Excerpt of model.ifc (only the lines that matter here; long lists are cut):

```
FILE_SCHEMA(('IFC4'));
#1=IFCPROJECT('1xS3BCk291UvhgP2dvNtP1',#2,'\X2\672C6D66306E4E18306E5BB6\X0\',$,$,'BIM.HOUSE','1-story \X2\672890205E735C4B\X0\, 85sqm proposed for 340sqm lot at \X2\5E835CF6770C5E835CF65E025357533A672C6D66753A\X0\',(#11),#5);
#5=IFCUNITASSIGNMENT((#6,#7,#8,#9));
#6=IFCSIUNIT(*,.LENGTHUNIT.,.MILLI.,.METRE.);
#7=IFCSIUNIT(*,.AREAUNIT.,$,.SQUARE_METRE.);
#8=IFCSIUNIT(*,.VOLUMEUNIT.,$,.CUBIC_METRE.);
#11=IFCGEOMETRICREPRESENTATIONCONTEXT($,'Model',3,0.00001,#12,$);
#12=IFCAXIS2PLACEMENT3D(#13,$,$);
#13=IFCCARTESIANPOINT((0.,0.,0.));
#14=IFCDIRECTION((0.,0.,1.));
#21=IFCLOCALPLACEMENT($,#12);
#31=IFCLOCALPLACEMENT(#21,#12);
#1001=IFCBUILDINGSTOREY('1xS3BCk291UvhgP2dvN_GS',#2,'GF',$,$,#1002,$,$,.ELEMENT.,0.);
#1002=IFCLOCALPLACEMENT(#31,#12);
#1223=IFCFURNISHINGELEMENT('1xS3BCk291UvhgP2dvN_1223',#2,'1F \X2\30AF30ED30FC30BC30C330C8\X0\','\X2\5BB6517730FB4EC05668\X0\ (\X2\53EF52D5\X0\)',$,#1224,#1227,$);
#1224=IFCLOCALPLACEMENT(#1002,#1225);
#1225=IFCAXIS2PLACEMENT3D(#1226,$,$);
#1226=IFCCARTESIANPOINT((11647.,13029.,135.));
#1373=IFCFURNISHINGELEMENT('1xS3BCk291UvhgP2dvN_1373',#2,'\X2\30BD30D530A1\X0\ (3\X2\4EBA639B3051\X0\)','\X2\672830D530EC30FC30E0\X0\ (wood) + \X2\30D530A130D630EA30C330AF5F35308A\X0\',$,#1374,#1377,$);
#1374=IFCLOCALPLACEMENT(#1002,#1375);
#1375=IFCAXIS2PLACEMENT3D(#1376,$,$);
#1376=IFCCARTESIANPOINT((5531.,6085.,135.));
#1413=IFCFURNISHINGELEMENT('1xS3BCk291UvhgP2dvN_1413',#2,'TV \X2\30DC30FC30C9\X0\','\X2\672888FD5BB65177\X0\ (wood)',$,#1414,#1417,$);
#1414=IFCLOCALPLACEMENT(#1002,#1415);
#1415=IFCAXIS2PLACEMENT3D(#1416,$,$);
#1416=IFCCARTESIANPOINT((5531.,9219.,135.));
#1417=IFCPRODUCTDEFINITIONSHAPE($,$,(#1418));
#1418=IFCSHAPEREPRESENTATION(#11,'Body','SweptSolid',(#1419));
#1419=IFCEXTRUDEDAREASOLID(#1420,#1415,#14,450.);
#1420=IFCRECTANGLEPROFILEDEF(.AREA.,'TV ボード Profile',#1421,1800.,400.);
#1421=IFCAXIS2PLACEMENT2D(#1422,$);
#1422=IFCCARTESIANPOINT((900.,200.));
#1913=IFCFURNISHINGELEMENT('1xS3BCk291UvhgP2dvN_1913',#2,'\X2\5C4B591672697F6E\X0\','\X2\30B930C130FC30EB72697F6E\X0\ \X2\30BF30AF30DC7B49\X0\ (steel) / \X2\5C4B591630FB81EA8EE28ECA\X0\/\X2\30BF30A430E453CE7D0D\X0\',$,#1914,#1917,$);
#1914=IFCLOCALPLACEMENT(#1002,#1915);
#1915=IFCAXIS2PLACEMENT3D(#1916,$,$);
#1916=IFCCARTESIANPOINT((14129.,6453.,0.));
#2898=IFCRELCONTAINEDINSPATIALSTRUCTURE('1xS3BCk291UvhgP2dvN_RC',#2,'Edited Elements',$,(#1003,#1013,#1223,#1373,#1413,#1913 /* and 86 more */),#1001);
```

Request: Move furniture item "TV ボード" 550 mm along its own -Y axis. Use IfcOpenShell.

```python
import ifcopenshell
import ifcopenshell.api.geometry
import ifcopenshell.util.placement
import ifcopenshell.util.unit

model = ifcopenshell.open("model.ifc")
unit_scale = ifcopenshell.util.unit.calculate_unit_scale(model)

item = model.by_guid("1xS3BCk291UvhgP2dvN_1413")
matrix = ifcopenshell.util.placement.get_local_placement(item.ObjectPlacement)
matrix[:3, 3] -= matrix[:3, 1] * 0.55 / unit_scale
ifcopenshell.api.geometry.edit_object_placement(model, product=item, matrix=matrix, is_si=False)

print(ifcopenshell.util.placement.get_local_placement(item.ObjectPlacement).round(3) + 0.0)

model.write("model_rev.ifc")
```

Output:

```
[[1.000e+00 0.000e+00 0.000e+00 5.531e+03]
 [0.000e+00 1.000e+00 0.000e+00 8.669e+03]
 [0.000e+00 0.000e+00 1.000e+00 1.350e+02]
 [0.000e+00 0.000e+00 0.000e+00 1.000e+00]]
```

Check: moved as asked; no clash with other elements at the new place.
